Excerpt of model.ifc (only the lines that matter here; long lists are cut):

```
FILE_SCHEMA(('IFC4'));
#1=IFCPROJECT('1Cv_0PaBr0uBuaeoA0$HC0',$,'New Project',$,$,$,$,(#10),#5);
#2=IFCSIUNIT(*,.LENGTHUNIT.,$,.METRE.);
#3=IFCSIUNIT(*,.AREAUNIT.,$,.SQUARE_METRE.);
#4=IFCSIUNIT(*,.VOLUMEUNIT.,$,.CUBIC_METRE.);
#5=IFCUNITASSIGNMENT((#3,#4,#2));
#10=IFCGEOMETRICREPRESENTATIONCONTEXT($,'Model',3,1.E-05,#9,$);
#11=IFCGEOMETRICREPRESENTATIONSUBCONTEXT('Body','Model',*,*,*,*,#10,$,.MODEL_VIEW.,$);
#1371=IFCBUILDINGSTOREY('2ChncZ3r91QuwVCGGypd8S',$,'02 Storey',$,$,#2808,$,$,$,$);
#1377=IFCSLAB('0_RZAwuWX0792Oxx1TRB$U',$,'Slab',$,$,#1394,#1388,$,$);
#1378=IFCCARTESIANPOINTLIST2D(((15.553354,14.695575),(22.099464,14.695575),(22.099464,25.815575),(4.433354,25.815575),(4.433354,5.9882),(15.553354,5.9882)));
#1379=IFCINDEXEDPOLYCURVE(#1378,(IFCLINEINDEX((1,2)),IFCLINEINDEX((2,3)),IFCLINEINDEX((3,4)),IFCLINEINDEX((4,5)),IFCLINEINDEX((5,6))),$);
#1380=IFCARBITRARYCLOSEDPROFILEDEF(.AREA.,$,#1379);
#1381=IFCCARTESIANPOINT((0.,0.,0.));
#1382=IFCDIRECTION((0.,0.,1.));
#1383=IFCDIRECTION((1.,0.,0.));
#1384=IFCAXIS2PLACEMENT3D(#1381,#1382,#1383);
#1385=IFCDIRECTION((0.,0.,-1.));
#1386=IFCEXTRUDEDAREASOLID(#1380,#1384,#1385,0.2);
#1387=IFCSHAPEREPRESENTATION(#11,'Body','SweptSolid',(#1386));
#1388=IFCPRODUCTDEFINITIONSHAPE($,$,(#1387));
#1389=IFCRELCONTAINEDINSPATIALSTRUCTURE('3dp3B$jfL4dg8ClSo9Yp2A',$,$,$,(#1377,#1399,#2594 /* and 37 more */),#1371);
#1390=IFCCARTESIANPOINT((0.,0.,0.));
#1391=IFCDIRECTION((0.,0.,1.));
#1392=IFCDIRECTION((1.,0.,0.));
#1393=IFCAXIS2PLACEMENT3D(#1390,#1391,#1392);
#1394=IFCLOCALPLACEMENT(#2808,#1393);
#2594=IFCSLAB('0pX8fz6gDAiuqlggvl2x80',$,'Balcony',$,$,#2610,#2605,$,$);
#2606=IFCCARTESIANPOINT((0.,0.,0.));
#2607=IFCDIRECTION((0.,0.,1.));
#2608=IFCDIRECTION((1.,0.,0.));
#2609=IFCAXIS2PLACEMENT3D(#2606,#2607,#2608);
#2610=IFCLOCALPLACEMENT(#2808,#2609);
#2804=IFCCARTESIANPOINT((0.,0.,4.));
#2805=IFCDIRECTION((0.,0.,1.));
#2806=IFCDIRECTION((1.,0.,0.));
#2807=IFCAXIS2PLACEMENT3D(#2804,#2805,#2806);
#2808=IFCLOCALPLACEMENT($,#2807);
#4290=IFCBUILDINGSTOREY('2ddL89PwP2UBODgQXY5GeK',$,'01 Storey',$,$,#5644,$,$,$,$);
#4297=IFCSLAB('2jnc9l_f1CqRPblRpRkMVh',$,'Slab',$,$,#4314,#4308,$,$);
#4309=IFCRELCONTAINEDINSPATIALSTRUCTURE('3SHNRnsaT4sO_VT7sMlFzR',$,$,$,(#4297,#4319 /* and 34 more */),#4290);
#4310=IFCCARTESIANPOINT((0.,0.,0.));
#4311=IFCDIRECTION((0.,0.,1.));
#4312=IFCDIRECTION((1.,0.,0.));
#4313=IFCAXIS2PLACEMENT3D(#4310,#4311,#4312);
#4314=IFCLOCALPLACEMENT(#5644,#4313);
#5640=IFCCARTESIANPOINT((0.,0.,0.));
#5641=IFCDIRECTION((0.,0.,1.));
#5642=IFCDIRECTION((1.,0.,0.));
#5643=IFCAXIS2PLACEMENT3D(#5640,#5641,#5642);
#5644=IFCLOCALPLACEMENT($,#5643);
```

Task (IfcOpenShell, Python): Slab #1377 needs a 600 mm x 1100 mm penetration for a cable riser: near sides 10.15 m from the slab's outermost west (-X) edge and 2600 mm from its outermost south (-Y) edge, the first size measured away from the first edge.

```python
import numpy as np
import ifcopenshell
import ifcopenshell.api.feature
import ifcopenshell.api.geometry
import ifcopenshell.api.root
import ifcopenshell.geom
import ifcopenshell.util.placement
import ifcopenshell.util.representation
import ifcopenshell.util.shape
import ifcopenshell.util.unit

model = ifcopenshell.open("model.ifc")
unit_scale = ifcopenshell.util.unit.calculate_unit_scale(model)
settings = ifcopenshell.geom.settings()


def volume(element):
    """Net volume in cubic metres, openings subtracted."""
    shape = ifcopenshell.geom.create_shape(settings, element)
    return ifcopenshell.util.shape.get_volume(shape.geometry)


slab = model.by_guid("0_RZAwuWX0792Oxx1TRB$U")
before = volume(slab)

# Extent in the slab's own axes, in metres. The edges named are its -X and -Y sides.
slab_shape = ifcopenshell.geom.create_shape(settings, slab)
vertices = ifcopenshell.util.shape.get_vertices(slab_shape.geometry)
x_min, y_min, bottom = vertices.min(axis=0)
top = vertices[:, 2].max()

opening = ifcopenshell.api.root.create_entity(model, ifc_class="IfcOpeningElement", name="Cable riser opening", predefined_type="OPENING")
context = ifcopenshell.util.representation.get_context(model, "Model", "Body", "MODEL_VIEW")
width, depth = 0.6, 1.1
outline = [(0.0, 0.0), (width, 0.0), (width, depth), (0.0, depth), (0.0, 0.0)]
# Overshoot both faces by 50 mm so the cut is clean.
shape = ifcopenshell.api.geometry.add_slab_representation(
    model, context=context, depth=top - bottom + 0.1, polyline=outline
)
ifcopenshell.api.geometry.assign_representation(model, product=opening, representation=shape)

matrix = ifcopenshell.util.placement.get_local_placement(slab.ObjectPlacement)
matrix[:, 3] = matrix @ np.append(np.array([x_min + 10.15, y_min + 2.6, bottom - 0.05]) / unit_scale, 1.0)
ifcopenshell.api.geometry.edit_object_placement(model, product=opening, matrix=matrix, is_si=False)
ifcopenshell.api.feature.add_feature(model, feature=opening, element=slab)

after = volume(slab)

print(f"slab volume {before:.3f} -> {after:.3f} m3")

model.write("model_updated.ifc")
```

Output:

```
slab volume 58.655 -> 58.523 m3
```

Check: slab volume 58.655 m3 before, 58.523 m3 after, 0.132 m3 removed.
